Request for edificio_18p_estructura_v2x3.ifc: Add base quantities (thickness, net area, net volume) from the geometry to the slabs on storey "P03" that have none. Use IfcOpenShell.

First a look at what the model holds.

```python
import ifcopenshell
import ifcopenshell.util.element
import ifcopenshell.util.unit

model = ifcopenshell.open("edificio_18p_estructura_v2x3.ifc")
print(model.schema)
for unit_type in ("LENGTHUNIT", "AREAUNIT", "VOLUMEUNIT"):
    print(unit_type, ifcopenshell.util.unit.calculate_unit_scale(model, unit_type))
storey = next(s for s in model.by_type("IfcBuildingStorey") if s.Name == "P03")
slabs = [e for e in ifcopenshell.util.element.get_decomposition(storey) if e.is_a("IfcSlab")]
for e in sorted(slabs, key=lambda e: e.id()):
    print(e.id(), e.is_a(), e.Name, list(ifcopenshell.util.element.get_psets(e, qtos_only=True)), sep=" | ")
```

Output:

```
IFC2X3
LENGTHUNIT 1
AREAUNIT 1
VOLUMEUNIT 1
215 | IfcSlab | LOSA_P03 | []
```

```python
import ifcopenshell
import ifcopenshell.api.pset
import ifcopenshell.geom
import ifcopenshell.util.element
import ifcopenshell.util.shape
import ifcopenshell.util.unit

model = ifcopenshell.open("edificio_18p_estructura_v2x3.ifc")
unit_scale = ifcopenshell.util.unit.calculate_unit_scale(model)
area_scale = ifcopenshell.util.unit.calculate_unit_scale(model, "AREAUNIT")
volume_scale = ifcopenshell.util.unit.calculate_unit_scale(model, "VOLUMEUNIT")
settings = ifcopenshell.geom.settings()

storey = next(s for s in model.by_type("IfcBuildingStorey") if s.Name == "P03")
slabs = [e for e in ifcopenshell.util.element.get_decomposition(storey) if e.is_a("IfcSlab")]

for e in sorted(slabs, key=lambda e: e.id()):
    if ifcopenshell.util.element.get_psets(e, qtos_only=True, should_inherit=False):
        continue
    # Geometry comes back in metres, in the element's own axes.
    shape = ifcopenshell.geom.create_shape(settings, e)
    values = {
        "Width": ifcopenshell.util.shape.get_z(shape.geometry) / unit_scale,
        "NetArea": ifcopenshell.util.shape.get_footprint_area(shape.geometry) / area_scale,
        "NetVolume": ifcopenshell.util.shape.get_volume(shape.geometry) / volume_scale,
    }
    qto = ifcopenshell.api.pset.add_qto(model, product=e, name="BaseQuantities")
    ifcopenshell.api.pset.edit_qto(model, qto=qto, properties=values)
    print(e.id(), {k: round(v, 3) for k, v in values.items()})

model.write("edificio_18p_estructura_v2x3_updated.ifc")
```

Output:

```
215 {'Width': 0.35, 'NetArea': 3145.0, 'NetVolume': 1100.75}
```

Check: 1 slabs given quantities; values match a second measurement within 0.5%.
